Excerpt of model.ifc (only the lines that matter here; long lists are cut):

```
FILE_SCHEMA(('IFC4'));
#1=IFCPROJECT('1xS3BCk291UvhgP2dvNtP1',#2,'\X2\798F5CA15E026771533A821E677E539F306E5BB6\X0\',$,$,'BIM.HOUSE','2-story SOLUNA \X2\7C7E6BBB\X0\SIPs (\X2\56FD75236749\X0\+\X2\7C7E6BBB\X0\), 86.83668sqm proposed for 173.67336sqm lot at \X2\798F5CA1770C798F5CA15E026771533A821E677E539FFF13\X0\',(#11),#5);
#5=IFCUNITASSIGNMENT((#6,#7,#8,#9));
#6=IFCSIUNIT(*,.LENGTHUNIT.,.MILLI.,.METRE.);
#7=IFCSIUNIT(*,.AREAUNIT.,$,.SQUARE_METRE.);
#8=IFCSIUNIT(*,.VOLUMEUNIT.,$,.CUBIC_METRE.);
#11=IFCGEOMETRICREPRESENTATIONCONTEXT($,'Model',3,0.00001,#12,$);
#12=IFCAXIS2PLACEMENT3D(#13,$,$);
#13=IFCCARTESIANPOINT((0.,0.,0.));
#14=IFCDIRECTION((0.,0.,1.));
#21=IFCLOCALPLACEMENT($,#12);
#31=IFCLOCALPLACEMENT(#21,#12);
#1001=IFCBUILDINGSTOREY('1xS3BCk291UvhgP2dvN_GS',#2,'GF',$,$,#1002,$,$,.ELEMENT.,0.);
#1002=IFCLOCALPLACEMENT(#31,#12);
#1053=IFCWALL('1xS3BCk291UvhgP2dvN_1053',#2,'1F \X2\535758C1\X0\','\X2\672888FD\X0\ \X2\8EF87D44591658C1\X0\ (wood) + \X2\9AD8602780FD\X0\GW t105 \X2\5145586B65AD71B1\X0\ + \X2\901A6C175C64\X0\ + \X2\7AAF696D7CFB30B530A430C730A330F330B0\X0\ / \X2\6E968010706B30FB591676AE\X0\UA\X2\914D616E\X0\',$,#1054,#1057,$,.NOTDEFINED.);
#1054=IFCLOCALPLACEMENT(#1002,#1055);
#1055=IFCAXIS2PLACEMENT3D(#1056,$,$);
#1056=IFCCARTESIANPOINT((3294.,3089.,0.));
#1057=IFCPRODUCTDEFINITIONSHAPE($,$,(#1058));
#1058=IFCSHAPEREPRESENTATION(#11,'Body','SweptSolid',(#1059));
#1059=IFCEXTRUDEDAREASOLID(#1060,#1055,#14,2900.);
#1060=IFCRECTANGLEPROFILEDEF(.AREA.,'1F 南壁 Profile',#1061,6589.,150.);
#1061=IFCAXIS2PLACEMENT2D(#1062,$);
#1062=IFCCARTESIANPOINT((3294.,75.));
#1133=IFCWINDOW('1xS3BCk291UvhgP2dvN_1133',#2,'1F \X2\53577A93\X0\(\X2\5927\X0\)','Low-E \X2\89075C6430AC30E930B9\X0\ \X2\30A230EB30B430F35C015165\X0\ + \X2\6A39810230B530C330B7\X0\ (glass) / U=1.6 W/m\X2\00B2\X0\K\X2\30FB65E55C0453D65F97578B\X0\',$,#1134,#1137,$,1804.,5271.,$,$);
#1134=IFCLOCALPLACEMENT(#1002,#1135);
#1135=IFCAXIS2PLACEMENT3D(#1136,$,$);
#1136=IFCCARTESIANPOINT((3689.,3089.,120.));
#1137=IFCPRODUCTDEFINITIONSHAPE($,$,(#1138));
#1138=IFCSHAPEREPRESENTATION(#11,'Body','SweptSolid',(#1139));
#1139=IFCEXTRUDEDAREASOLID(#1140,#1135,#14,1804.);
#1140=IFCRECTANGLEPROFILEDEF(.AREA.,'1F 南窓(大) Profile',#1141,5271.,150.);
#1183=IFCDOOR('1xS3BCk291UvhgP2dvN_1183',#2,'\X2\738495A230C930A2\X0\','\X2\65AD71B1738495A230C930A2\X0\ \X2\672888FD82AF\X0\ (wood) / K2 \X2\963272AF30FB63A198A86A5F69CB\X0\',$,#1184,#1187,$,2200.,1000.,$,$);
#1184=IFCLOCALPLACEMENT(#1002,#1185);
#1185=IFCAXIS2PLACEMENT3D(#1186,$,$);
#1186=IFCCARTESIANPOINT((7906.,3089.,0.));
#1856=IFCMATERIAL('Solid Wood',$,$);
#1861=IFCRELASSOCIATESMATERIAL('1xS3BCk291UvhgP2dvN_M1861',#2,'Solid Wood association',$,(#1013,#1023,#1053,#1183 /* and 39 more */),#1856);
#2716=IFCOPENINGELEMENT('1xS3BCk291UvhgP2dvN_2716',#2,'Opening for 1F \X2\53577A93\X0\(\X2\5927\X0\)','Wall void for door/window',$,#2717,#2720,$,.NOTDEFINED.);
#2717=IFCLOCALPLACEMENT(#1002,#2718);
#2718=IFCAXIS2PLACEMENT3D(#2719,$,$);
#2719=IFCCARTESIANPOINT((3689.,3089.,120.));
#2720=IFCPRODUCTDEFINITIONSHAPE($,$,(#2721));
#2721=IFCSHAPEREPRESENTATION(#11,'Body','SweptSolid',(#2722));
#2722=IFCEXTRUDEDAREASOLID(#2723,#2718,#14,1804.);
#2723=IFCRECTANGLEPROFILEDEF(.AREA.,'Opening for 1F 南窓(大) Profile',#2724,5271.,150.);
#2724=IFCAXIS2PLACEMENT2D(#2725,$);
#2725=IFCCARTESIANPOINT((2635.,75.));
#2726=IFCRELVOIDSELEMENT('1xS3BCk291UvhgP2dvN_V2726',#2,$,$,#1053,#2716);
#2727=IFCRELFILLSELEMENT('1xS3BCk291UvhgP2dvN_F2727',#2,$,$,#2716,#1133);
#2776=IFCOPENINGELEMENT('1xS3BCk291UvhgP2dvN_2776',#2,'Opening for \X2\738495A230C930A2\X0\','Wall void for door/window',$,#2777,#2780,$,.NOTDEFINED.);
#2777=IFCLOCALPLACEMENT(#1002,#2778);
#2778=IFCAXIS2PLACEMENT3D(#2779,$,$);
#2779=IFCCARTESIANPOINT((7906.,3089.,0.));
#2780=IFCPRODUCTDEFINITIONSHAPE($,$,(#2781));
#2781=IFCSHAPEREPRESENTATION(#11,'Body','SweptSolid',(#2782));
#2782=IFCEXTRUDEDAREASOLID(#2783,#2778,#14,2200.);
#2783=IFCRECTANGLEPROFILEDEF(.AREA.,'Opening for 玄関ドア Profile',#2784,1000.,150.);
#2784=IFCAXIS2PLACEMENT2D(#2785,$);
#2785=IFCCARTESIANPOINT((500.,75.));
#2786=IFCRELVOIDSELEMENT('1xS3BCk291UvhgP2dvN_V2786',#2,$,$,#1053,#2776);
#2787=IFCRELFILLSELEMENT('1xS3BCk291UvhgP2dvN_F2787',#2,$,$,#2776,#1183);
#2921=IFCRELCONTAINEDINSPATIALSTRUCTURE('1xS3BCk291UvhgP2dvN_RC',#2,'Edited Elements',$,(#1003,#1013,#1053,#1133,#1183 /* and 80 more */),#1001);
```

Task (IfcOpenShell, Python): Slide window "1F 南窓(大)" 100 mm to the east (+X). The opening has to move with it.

```python
import ifcopenshell
import ifcopenshell.api.geometry
import ifcopenshell.util.placement

model = ifcopenshell.open("model.ifc")

window = model.by_id(1133)
opening = window.FillsVoids[0].RelatingOpeningElement
wall = opening.VoidsElements[0].RelatingBuildingElement

wall_matrix = ifcopenshell.util.placement.get_local_placement(wall.ObjectPlacement)
shift = wall_matrix[:3, 0] * 100.0
before = ifcopenshell.util.placement.get_local_placement(window.ObjectPlacement)[:3, 3].copy()

# The window is not placed relative to its opening, so move both.
for product in (opening, window):
    matrix = ifcopenshell.util.placement.get_local_placement(product.ObjectPlacement)
    matrix[:3, 3] += shift
    ifcopenshell.api.geometry.edit_object_placement(model, product=product, matrix=matrix, is_si=False)

after = ifcopenshell.util.placement.get_local_placement(window.ObjectPlacement)[:3, 3]
print("window moved by", (after - before).round(3) + 0.0)

model.write("model_updated.ifc")
```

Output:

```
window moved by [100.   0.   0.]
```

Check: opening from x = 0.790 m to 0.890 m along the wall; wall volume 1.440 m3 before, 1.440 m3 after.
